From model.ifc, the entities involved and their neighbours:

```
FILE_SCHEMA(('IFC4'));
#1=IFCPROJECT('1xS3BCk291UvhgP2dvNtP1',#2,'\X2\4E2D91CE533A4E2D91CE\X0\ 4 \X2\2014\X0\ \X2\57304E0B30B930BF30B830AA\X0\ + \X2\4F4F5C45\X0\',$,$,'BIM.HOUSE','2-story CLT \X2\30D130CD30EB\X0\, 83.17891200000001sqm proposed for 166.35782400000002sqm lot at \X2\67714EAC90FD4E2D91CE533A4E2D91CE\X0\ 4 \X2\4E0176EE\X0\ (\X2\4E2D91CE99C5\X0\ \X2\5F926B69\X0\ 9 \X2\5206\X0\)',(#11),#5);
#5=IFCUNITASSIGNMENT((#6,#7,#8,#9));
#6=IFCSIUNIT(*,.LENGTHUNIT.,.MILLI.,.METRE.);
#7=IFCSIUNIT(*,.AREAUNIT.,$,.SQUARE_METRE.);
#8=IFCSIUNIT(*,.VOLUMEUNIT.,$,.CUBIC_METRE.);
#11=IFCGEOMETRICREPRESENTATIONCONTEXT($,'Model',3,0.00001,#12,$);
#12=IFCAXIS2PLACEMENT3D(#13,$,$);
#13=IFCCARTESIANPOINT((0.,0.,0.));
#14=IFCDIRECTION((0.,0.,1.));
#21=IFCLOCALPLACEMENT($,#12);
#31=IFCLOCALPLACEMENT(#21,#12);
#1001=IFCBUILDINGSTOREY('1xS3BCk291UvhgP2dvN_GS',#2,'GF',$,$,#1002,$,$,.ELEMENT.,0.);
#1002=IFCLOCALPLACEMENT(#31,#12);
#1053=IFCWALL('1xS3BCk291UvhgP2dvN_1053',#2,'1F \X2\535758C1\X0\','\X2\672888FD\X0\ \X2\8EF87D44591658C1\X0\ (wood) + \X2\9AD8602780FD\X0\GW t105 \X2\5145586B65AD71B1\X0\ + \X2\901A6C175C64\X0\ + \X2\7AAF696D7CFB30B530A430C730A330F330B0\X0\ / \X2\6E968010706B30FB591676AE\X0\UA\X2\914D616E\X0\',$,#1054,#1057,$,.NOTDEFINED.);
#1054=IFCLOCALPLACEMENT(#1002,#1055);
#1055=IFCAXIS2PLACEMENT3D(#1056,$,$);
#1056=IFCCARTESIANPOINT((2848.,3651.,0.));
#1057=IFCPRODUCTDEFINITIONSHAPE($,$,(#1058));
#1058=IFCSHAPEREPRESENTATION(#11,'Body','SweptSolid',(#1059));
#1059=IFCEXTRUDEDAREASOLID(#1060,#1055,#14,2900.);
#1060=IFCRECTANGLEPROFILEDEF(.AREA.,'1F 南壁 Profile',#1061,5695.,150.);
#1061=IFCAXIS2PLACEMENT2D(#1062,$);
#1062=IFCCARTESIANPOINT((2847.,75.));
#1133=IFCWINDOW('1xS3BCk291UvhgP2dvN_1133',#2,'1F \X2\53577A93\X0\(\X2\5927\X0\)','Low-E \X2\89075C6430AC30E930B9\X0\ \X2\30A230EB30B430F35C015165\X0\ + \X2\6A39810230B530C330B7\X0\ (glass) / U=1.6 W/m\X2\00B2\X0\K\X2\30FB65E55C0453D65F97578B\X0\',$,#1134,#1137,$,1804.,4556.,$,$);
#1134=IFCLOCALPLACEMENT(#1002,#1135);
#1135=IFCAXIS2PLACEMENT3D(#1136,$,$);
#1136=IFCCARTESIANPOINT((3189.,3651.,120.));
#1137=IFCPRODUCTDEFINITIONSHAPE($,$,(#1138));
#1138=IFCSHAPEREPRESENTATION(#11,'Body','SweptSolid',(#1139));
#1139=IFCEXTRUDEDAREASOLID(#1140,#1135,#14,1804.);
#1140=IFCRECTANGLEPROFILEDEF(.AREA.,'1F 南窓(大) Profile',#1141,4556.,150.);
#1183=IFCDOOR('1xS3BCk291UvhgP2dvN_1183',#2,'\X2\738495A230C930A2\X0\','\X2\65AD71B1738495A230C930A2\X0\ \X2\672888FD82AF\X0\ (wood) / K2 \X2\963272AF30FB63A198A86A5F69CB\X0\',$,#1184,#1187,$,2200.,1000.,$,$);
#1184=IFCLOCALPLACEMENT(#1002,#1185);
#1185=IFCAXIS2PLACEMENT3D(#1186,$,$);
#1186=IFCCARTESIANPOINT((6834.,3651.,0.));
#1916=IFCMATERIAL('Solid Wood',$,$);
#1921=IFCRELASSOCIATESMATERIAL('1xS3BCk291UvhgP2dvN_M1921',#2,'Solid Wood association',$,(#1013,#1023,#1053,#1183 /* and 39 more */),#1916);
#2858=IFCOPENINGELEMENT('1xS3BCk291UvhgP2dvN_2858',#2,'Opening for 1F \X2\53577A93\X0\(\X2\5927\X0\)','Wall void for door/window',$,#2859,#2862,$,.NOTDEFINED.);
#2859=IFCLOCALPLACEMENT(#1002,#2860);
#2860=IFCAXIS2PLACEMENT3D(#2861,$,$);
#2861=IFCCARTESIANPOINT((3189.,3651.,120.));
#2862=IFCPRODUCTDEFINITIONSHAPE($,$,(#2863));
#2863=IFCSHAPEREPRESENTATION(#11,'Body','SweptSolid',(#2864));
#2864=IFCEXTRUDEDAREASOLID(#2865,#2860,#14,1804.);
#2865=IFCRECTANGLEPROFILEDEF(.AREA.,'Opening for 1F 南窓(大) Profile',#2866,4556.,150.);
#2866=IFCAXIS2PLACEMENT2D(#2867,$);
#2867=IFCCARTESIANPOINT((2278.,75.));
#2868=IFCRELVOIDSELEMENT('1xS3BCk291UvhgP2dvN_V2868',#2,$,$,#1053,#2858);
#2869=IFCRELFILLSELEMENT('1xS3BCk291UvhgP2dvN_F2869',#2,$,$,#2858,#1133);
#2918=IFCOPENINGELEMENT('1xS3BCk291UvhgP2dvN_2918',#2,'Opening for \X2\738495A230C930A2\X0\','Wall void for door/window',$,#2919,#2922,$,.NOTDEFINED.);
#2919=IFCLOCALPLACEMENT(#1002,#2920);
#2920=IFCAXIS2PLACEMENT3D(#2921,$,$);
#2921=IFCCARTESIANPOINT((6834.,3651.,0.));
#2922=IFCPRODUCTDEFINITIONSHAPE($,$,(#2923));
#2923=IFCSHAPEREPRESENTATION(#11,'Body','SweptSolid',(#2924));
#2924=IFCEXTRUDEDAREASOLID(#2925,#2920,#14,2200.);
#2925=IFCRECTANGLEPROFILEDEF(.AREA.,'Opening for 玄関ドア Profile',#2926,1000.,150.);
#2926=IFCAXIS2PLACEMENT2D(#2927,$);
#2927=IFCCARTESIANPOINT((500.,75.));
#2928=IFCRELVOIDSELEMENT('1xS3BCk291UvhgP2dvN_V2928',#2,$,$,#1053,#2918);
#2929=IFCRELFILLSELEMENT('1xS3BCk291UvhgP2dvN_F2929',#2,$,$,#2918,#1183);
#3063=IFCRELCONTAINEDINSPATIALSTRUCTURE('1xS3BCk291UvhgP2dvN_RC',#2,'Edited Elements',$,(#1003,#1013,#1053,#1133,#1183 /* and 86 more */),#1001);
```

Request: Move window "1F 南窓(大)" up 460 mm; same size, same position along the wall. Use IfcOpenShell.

```python
import numpy as np
import ifcopenshell
import ifcopenshell.api.geometry
import ifcopenshell.util.placement
import ifcopenshell.util.unit

model = ifcopenshell.open("model.ifc")
unit_scale = ifcopenshell.util.unit.calculate_unit_scale(model)

window = model.by_id(1133)
opening = window.FillsVoids[0].RelatingOpeningElement
dz = 0.46 / unit_scale

shift = np.array([0.0, 0.0, dz])
# The window is not placed relative to its opening, so move both.
for product in (opening, window):
    matrix = ifcopenshell.util.placement.get_local_placement(product.ObjectPlacement)
    matrix[:3, 3] += shift
    ifcopenshell.api.geometry.edit_object_placement(model, product=product, matrix=matrix, is_si=False)

print(f"moved by {dz * unit_scale:+.3f} m")

model.write("model_rev.ifc")
```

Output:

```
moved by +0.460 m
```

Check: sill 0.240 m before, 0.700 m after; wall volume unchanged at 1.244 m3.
